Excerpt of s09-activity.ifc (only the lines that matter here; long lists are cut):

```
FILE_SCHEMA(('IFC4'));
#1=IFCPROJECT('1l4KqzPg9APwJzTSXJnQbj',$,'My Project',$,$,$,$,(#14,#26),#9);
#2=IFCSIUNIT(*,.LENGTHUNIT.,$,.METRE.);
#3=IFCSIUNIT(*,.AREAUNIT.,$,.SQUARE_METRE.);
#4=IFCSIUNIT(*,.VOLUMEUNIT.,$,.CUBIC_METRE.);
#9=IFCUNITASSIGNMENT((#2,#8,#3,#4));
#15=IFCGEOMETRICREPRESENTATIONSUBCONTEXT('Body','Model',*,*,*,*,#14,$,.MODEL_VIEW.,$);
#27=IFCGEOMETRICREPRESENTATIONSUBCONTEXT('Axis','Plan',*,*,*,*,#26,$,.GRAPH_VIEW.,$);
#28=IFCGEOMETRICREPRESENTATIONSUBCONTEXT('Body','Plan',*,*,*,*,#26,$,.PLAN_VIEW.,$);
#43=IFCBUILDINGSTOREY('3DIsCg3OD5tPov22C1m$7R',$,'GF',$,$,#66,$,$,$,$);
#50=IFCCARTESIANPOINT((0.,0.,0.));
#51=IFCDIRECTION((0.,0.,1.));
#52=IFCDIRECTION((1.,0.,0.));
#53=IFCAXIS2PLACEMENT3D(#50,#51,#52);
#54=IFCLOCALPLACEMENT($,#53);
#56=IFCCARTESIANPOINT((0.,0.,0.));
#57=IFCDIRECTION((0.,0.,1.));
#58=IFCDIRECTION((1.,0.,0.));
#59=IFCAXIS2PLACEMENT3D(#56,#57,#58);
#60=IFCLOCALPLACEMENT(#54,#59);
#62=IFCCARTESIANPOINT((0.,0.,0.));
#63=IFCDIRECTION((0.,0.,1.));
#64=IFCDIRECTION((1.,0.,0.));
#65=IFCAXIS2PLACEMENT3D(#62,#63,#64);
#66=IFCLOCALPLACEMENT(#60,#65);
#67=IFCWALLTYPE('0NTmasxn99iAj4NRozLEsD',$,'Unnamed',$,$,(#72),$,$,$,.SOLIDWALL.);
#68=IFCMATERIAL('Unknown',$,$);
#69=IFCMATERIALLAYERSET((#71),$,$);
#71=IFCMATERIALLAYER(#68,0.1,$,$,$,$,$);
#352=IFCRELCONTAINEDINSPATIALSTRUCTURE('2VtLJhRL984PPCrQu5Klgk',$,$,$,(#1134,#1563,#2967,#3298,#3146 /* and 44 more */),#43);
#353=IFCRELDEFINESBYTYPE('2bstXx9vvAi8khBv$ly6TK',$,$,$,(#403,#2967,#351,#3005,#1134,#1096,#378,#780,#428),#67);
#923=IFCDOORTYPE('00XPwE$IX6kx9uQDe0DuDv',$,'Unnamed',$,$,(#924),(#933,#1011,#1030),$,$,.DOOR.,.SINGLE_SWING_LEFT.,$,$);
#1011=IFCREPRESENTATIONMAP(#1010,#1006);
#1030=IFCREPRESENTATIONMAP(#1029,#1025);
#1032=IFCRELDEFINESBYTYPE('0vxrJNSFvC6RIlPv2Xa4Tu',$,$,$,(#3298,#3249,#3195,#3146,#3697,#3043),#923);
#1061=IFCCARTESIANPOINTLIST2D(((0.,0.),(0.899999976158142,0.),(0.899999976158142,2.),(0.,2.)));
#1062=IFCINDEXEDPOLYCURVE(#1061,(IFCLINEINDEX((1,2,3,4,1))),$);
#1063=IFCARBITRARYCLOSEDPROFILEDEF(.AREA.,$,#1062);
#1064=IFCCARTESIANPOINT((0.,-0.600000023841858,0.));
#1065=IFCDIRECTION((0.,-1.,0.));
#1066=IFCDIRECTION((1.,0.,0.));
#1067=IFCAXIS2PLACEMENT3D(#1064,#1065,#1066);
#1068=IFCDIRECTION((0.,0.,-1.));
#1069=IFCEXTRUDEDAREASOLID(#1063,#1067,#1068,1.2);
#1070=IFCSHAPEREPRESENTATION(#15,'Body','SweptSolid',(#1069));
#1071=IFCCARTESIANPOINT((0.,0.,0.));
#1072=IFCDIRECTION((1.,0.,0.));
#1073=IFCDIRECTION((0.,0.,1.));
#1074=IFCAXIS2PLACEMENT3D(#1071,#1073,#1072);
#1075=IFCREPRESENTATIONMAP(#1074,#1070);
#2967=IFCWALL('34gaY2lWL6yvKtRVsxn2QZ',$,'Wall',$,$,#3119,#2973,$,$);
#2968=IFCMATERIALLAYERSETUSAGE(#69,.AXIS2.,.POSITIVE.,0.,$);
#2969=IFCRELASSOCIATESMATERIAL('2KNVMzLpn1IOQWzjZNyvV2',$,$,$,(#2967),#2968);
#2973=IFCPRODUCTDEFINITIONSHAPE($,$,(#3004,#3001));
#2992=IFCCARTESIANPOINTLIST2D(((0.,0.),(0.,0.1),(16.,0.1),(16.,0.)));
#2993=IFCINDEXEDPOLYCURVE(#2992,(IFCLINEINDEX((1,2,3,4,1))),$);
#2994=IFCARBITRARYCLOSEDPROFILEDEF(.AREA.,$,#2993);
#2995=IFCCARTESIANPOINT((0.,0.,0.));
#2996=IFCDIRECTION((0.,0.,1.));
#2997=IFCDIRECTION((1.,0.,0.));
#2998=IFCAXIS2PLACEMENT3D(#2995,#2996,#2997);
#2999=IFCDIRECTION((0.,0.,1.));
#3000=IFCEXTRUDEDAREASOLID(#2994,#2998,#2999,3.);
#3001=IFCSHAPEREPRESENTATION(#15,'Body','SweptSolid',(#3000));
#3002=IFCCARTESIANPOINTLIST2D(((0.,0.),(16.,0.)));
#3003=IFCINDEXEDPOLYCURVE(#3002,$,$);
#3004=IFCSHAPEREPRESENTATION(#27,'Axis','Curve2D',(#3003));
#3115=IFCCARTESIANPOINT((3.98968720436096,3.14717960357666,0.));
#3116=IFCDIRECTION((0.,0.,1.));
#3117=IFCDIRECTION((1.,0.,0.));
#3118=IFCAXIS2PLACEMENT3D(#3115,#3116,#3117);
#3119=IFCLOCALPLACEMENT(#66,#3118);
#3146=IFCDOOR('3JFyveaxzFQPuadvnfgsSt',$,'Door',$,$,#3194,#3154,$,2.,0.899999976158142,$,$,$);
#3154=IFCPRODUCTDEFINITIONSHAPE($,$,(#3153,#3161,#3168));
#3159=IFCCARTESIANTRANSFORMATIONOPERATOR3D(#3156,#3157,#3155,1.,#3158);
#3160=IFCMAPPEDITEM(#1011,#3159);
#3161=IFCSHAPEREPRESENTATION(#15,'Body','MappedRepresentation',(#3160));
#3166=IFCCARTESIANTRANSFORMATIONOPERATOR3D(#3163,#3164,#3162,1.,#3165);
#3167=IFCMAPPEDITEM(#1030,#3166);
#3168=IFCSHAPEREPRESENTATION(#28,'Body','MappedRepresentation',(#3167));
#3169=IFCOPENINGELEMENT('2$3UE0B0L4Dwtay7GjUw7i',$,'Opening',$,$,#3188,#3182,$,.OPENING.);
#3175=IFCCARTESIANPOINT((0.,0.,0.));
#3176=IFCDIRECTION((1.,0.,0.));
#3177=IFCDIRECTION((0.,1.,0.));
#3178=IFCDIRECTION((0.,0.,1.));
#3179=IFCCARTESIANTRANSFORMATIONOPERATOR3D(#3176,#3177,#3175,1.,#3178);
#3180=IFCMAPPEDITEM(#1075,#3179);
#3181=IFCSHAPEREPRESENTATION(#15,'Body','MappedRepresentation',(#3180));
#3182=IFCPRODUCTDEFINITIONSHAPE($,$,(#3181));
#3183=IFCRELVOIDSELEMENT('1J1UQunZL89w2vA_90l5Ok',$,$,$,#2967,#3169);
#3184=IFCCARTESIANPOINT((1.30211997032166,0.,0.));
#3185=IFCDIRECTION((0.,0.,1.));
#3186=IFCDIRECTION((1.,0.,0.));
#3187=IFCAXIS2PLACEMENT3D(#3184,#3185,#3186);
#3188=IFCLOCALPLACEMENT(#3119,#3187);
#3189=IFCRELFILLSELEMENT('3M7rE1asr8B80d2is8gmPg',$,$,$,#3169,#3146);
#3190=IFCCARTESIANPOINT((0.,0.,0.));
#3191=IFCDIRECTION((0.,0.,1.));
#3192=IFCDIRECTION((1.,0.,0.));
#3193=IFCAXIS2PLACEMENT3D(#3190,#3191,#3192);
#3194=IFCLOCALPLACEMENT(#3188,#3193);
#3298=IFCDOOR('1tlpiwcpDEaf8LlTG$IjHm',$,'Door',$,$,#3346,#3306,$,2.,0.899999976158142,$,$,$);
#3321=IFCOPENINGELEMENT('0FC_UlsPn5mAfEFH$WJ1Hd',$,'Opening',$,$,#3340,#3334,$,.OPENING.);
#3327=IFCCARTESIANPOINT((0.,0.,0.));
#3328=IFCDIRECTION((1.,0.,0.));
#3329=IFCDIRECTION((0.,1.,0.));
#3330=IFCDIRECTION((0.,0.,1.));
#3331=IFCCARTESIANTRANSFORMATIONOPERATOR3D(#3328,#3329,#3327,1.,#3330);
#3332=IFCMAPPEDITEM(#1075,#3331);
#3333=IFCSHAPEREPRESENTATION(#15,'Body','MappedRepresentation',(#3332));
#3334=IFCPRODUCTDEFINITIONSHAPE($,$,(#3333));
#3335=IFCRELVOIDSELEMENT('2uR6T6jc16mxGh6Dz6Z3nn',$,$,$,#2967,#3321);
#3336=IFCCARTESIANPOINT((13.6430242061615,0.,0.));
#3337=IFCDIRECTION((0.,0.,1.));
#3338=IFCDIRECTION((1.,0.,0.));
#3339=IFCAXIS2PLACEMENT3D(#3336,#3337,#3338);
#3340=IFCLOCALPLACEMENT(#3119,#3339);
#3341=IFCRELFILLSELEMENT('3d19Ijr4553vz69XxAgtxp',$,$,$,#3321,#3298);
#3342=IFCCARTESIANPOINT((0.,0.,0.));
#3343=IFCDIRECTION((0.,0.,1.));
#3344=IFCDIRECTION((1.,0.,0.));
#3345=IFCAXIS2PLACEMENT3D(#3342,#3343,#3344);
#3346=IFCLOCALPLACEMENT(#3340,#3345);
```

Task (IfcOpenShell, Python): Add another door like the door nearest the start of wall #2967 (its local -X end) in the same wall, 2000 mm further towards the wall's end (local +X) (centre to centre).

```python
import ifcopenshell
import ifcopenshell.api.feature
import ifcopenshell.api.geometry
import ifcopenshell.api.root
import ifcopenshell.geom
import ifcopenshell.util.element
import ifcopenshell.util.placement
import ifcopenshell.util.shape
import ifcopenshell.util.unit

model = ifcopenshell.open("s09-activity.ifc")
unit_scale = ifcopenshell.util.unit.calculate_unit_scale(model)
settings = ifcopenshell.geom.settings()


def volume(element):
    """Net volume in cubic metres, openings subtracted."""
    shape = ifcopenshell.geom.create_shape(settings, element)
    return ifcopenshell.util.shape.get_volume(shape.geometry)


door = model.by_guid("3JFyveaxzFQPuadvnfgsSt")
opening = door.FillsVoids[0].RelatingOpeningElement
wall = opening.VoidsElements[0].RelatingBuildingElement
before = volume(wall)
shift = ifcopenshell.util.placement.get_local_placement(wall.ObjectPlacement)[:3, 0] * 2 / unit_scale

# copy_class copies the void relationship, type, container and properties, but no geometry.
new_opening = ifcopenshell.api.root.copy_class(model, product=opening)
new_opening.Representation = ifcopenshell.util.element.copy_deep(
    model, opening.Representation, exclude=["IfcGeometricRepresentationContext", "IfcRepresentationMap"]
)
new_door = ifcopenshell.api.root.copy_class(model, product=door)
new_door.Representation = ifcopenshell.util.element.copy_deep(
    model, door.Representation, exclude=["IfcGeometricRepresentationContext", "IfcRepresentationMap"]
)
ifcopenshell.api.feature.add_filling(model, opening=new_opening, element=new_door)

for old, new in ((opening, new_opening), (door, new_door)):
    matrix = ifcopenshell.util.placement.get_local_placement(old.ObjectPlacement)
    matrix[:3, 3] += shift
    ifcopenshell.api.geometry.edit_object_placement(model, product=new, matrix=matrix, is_si=False)

after = volume(wall)

print(f"wall volume {before:.3f} -> {after:.3f} m3")

model.write("s09-activity_v2.ifc")
```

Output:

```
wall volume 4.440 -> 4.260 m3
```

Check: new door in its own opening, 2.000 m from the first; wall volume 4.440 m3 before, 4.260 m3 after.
